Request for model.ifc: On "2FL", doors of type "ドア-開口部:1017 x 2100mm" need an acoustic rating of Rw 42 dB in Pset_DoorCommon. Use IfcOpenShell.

First a look at what the model holds.

```python
import ifcopenshell
import ifcopenshell.util.element

model = ifcopenshell.open("model.ifc")
print(model.schema)
storey = next(s for s in model.by_type("IfcBuildingStorey") if s.Name == "2FL")
doors = [e for e in ifcopenshell.util.element.get_decomposition(storey) if e.is_a("IfcDoor")]
seen = {}
for e in doors:
    element_type = ifcopenshell.util.element.get_type(e)
    key = (element_type.Name if element_type != e and element_type else None, ifcopenshell.util.element.get_pset(e, "Pset_DoorCommon", "AcousticRating"))
    seen[key] = seen.get(key, 0) + 1
for (name, value), count in sorted(seen.items(), key=str):
    print(count, "x", name, "|", value)
```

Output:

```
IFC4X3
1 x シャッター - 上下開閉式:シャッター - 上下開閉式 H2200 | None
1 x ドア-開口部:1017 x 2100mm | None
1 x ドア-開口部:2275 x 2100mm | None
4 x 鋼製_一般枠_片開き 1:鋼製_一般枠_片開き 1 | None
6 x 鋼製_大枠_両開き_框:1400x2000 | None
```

```python
import ifcopenshell
import ifcopenshell.api.pset
import ifcopenshell.util.element

model = ifcopenshell.open("model.ifc")

storey = next(s for s in model.by_type("IfcBuildingStorey") if s.Name == "2FL")
doors = [e for e in ifcopenshell.util.element.get_decomposition(storey) if e.is_a("IfcDoor")]

count = 0
for e in doors:
    element_type = ifcopenshell.util.element.get_type(e)
    if element_type in (None, e) or element_type.Name != "ドア-開口部:1017 x 2100mm":
        continue
    # add_pset returns the element's existing set when there is one.
    pset = ifcopenshell.api.pset.add_pset(model, product=e, name="Pset_DoorCommon")
    ifcopenshell.api.pset.edit_pset(model, pset=pset, properties={"AcousticRating": "Rw 42 dB"})
    count += 1

print(count, "doors updated")

model.write("model_updated.ifc")
```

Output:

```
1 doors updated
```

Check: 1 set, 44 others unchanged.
